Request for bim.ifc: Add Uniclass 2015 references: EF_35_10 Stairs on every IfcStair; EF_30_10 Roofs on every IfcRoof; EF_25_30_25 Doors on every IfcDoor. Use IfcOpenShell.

First a look at what the model holds.

```python
import ifcopenshell

model = ifcopenshell.open("bim.ifc")
print(model.schema)
print("classifications:", [c.Name for c in model.by_type("IfcClassification")])
for ifc_class in ("IfcDoor", "IfcRoof", "IfcStair", "IfcWall", "IfcWindow"):
    print(ifc_class, len(model.by_type(ifc_class)))
```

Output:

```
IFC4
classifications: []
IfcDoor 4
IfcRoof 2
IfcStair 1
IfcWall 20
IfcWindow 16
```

```python
import ifcopenshell
import ifcopenshell.api.classification

model = ifcopenshell.open("bim.ifc")

system = ifcopenshell.api.classification.add_classification(model, classification="Uniclass 2015")

codes = {
    "IfcStair": ("EF_35_10", "Stairs"),
    "IfcRoof": ("EF_30_10", "Roofs"),
    "IfcDoor": ("EF_25_30_25", "Doors"),
}
for ifc_class, (code, name) in codes.items():
    products = model.by_type(ifc_class)
    ifcopenshell.api.classification.add_reference(
        model, products=products, classification=system, identification=code, name=name
    )
    print(code, len(products))

model.write("bim_updated.ifc")
```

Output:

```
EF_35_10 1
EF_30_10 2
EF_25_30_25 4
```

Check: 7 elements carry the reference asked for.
